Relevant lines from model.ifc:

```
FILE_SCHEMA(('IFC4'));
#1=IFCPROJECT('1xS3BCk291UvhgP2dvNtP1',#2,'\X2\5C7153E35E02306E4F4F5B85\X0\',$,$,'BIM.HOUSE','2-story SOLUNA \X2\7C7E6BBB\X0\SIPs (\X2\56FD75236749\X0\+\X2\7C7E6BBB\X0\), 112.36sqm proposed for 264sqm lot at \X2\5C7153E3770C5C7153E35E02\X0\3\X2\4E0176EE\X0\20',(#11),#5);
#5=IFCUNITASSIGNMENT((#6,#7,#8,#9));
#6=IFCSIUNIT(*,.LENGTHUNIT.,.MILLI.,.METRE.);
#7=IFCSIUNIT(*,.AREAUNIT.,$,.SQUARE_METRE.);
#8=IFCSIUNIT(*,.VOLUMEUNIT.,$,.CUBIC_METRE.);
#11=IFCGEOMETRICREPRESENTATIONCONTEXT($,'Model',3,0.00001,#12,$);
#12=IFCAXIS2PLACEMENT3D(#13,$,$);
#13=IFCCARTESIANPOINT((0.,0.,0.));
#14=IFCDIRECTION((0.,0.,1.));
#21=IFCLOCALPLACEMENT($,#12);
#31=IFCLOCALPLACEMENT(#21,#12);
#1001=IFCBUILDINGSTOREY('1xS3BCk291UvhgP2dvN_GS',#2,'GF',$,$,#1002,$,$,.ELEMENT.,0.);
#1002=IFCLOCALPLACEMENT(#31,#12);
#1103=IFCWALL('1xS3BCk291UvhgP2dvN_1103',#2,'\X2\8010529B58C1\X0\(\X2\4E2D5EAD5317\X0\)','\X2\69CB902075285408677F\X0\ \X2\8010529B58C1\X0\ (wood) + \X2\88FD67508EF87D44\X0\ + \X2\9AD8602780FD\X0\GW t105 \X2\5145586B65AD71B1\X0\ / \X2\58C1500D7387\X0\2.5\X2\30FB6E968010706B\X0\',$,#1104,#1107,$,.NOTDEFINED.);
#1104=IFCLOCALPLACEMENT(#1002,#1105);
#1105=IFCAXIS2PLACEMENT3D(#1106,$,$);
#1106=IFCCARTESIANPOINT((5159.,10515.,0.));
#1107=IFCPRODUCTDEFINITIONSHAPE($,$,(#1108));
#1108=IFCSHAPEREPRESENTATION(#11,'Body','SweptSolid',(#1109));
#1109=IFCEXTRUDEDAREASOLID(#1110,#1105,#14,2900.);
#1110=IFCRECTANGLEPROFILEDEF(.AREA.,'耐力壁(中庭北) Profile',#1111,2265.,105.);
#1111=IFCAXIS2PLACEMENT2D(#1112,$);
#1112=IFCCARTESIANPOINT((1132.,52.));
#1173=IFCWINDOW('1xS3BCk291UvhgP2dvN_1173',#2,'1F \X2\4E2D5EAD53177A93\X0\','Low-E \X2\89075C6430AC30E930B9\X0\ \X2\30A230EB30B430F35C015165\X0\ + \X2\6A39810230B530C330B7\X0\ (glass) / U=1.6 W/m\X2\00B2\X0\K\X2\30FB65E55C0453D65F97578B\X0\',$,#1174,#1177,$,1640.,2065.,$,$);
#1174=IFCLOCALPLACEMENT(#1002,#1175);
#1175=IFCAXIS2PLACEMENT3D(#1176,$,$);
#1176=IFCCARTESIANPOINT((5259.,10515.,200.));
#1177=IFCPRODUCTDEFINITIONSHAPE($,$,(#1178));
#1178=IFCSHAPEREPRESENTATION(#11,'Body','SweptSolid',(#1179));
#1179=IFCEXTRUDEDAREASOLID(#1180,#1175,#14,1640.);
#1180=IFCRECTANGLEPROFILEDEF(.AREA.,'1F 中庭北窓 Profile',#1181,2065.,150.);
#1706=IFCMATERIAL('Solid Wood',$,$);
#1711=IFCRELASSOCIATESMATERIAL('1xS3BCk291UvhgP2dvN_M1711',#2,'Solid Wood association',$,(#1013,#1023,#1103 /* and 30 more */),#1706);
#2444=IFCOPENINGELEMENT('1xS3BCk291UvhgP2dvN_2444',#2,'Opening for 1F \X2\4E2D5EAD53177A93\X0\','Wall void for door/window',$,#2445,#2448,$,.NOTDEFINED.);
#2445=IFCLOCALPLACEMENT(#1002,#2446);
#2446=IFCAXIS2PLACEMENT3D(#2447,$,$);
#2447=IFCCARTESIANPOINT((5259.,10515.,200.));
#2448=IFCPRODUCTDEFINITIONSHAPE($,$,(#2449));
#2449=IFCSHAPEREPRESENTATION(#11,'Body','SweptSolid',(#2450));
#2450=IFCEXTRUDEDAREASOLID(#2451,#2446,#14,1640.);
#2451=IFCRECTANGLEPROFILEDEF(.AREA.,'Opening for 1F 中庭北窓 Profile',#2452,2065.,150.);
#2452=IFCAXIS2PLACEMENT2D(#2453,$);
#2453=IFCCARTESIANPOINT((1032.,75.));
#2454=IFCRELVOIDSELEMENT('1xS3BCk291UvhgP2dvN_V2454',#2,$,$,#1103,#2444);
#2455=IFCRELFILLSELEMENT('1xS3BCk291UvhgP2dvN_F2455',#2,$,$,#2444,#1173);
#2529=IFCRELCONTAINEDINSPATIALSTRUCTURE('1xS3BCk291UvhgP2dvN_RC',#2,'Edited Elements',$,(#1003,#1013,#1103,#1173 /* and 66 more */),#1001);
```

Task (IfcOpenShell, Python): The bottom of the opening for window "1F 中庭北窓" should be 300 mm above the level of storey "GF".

```python
import numpy as np
import ifcopenshell
import ifcopenshell.api.geometry
import ifcopenshell.geom
import ifcopenshell.util.element
import ifcopenshell.util.placement
import ifcopenshell.util.shape
import ifcopenshell.util.unit

model = ifcopenshell.open("model.ifc")
unit_scale = ifcopenshell.util.unit.calculate_unit_scale(model)

window = model.by_id(1173)
opening = window.FillsVoids[0].RelatingOpeningElement
storey = ifcopenshell.util.element.get_container(window, ifc_class="IfcBuildingStorey")
level = ifcopenshell.util.placement.get_local_placement(storey.ObjectPlacement)[2, 3]

# The opening's origin need not be at the sill, so measure its lowest point.
shape = ifcopenshell.geom.create_shape(ifcopenshell.geom.settings(), opening)
bottom = ifcopenshell.util.shape.get_shape_bottom_elevation(shape, shape.geometry) / unit_scale
dz = level + 0.3 / unit_scale - bottom

shift = np.array([0.0, 0.0, dz])
# The window is not placed relative to its opening, so move both.
for product in (opening, window):
    matrix = ifcopenshell.util.placement.get_local_placement(product.ObjectPlacement)
    matrix[:3, 3] += shift
    ifcopenshell.api.geometry.edit_object_placement(model, product=product, matrix=matrix, is_si=False)

print(f"moved by {dz * unit_scale:+.3f} m")

model.write("model_edited.ifc")
```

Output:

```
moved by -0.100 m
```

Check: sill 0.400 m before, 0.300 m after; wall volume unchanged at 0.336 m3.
